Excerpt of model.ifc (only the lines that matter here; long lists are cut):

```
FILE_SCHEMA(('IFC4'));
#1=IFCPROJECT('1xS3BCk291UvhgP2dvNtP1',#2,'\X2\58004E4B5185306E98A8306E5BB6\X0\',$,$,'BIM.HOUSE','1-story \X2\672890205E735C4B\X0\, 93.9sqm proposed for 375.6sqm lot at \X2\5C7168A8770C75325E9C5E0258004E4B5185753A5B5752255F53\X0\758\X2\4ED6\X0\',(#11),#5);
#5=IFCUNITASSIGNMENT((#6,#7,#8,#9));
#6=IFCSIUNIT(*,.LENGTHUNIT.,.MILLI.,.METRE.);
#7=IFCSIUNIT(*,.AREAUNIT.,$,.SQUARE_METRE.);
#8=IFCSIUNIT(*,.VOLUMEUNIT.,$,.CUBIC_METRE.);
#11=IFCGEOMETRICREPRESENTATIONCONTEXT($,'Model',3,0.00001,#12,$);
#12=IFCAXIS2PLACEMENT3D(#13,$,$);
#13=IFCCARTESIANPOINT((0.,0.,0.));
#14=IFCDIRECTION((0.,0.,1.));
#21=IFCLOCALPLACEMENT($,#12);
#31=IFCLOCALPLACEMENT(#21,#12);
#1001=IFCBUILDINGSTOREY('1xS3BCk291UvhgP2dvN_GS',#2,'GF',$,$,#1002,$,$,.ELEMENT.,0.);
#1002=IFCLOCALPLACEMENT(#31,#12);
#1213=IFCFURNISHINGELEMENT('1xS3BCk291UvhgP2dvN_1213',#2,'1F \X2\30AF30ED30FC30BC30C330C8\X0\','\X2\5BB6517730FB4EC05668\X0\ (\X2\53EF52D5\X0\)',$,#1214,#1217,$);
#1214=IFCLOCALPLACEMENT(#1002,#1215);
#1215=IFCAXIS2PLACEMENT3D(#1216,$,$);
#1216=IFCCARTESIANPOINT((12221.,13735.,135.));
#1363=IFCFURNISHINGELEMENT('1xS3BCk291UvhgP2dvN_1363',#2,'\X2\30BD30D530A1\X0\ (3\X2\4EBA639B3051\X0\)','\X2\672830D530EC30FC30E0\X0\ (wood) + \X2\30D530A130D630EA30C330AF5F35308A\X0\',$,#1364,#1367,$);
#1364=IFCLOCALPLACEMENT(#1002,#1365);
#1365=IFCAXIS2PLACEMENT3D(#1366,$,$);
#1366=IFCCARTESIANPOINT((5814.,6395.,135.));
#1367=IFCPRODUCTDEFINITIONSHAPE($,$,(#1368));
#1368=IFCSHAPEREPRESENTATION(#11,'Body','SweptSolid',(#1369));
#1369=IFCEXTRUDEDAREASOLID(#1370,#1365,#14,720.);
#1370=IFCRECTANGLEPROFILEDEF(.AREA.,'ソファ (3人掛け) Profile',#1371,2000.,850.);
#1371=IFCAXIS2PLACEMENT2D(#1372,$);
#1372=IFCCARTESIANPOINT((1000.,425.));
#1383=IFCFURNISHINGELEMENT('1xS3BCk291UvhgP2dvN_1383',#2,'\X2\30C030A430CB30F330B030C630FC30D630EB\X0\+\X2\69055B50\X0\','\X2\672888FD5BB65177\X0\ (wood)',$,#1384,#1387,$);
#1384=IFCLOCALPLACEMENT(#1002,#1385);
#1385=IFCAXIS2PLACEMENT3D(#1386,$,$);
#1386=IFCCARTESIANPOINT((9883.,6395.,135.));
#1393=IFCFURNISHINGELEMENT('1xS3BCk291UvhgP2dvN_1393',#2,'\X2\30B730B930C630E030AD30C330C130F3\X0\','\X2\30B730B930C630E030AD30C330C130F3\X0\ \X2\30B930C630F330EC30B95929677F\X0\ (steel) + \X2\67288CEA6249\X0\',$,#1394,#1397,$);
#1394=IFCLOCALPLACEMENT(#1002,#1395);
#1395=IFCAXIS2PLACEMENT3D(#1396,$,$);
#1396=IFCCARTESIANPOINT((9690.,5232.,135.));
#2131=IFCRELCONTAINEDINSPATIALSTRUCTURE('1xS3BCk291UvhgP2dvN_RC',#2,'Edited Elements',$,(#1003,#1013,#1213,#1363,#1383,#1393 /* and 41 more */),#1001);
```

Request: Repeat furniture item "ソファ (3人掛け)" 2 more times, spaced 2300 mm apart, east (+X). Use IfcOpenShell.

```python
import numpy as np
import ifcopenshell
import ifcopenshell.api.geometry
import ifcopenshell.api.root
import ifcopenshell.util.element
import ifcopenshell.util.placement

model = ifcopenshell.open("model.ifc")


def reuse_history(source, copy):
    """copy_class also copies each property set's owner history, people and application; keep the originals."""
    for rel in copy.IsDefinedBy:
        if rel.is_a("IfcRelDefinesByProperties") and (history := rel.RelatingPropertyDefinition.OwnerHistory):
            rel.RelatingPropertyDefinition.OwnerHistory = source.OwnerHistory
            ifcopenshell.util.element.remove_deep2(model, history)


source = model.by_guid("1xS3BCk291UvhgP2dvN_1363")
base = ifcopenshell.util.placement.get_local_placement(source.ObjectPlacement)
step = np.array([1.0, 0.0, 0.0]) * 2300.0

for i in range(1, 3):
    copy = ifcopenshell.api.root.copy_class(model, product=source)
    copy.Representation = ifcopenshell.util.element.copy_deep(
        model, source.Representation, exclude=["IfcGeometricRepresentationContext", "IfcRepresentationMap"]
    )
    reuse_history(source, copy)
    matrix = base.copy()
    matrix[:3, 3] += i * step
    print("added at", matrix[:3, 3].round(3) + 0.0)
    ifcopenshell.api.geometry.edit_object_placement(model, product=copy, matrix=matrix, is_si=False)

model.write("model_rev.ifc")
```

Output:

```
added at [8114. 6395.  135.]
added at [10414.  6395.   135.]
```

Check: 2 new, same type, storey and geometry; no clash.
